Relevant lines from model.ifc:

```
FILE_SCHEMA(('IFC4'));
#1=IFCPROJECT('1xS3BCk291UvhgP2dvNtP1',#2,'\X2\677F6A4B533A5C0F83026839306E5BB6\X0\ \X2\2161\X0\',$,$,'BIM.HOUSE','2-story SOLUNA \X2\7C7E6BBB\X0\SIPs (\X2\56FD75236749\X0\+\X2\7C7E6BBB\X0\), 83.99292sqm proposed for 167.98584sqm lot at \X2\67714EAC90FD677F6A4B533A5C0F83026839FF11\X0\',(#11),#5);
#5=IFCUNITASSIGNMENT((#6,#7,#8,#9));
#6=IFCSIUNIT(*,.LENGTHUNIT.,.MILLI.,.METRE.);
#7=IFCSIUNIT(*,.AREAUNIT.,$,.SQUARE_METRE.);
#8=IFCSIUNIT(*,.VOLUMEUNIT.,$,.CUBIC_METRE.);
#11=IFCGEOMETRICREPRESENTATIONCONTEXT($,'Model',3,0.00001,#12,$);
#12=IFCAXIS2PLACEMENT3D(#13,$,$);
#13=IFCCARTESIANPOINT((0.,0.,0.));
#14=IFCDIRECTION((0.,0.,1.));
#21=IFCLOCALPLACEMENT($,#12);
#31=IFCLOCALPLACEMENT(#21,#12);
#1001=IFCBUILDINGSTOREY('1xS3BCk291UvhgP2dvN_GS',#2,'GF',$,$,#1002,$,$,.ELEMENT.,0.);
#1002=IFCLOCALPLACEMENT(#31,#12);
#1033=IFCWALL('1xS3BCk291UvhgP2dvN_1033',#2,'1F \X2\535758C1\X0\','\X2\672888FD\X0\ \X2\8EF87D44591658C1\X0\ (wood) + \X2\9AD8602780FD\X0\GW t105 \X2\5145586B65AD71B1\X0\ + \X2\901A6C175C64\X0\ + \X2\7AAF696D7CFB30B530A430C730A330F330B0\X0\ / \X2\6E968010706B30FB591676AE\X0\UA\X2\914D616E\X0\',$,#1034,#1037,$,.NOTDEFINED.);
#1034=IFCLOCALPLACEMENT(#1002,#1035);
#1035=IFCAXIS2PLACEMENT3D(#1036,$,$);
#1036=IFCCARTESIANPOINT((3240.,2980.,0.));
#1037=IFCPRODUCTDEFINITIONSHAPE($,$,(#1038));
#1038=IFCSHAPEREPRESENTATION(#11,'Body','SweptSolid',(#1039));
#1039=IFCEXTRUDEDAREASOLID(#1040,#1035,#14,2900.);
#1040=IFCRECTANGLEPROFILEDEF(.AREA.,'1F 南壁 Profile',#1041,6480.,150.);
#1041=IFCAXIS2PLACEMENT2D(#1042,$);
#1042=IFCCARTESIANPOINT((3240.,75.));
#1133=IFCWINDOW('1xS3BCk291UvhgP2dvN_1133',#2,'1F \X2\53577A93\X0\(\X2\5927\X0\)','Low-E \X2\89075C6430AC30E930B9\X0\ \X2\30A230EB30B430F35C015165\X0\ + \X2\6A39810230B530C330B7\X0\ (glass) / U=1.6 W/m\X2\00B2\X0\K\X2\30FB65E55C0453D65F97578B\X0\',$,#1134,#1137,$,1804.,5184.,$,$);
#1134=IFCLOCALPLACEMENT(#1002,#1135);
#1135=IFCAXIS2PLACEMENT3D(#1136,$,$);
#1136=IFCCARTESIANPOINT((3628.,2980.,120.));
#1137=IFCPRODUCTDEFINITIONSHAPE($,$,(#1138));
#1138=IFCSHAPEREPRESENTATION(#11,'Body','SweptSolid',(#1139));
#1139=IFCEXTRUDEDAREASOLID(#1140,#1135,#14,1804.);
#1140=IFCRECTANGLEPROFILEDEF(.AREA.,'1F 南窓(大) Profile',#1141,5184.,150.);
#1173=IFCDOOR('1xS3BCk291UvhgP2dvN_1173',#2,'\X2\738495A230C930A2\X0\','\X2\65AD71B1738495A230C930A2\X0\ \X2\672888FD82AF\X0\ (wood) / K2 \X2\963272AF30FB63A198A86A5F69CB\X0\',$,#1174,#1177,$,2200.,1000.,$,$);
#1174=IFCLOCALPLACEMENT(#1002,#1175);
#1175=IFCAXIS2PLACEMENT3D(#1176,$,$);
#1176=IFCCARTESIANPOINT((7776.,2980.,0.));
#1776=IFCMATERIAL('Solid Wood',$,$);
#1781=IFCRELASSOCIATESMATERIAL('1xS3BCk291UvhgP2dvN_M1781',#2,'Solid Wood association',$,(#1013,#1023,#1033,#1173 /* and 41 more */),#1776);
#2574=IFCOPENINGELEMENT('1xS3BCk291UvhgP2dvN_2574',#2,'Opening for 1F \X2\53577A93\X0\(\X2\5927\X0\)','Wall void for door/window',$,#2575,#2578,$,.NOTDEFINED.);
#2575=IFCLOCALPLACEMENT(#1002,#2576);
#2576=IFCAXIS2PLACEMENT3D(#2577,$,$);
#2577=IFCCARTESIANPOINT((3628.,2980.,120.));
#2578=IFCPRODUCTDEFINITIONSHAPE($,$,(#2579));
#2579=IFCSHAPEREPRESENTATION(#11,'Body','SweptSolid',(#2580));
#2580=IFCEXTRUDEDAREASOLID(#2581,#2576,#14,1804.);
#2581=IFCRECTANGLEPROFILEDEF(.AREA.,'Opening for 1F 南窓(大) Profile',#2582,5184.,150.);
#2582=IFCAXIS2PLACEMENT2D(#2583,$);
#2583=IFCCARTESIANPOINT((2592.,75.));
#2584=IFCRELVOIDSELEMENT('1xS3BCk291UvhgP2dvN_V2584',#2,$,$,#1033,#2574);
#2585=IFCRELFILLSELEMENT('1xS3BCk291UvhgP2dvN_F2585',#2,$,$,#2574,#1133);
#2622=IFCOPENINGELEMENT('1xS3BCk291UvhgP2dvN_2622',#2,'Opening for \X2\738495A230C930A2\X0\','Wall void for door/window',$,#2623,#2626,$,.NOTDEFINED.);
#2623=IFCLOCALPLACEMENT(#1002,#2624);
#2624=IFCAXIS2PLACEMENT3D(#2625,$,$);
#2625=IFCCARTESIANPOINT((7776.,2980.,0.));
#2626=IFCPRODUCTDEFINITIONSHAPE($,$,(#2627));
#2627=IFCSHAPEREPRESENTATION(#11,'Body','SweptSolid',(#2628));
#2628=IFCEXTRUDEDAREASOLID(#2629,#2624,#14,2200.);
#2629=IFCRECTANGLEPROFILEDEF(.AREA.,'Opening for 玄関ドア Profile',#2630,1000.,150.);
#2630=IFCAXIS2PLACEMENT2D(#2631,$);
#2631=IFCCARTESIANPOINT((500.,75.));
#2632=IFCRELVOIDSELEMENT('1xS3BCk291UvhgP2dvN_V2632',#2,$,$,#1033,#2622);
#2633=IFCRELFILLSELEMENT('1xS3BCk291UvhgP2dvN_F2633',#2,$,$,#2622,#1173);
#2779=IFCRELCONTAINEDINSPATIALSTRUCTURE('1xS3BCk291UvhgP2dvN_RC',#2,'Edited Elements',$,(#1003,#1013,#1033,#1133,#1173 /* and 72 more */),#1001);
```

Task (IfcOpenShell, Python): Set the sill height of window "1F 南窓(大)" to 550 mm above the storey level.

```python
import numpy as np
import ifcopenshell
import ifcopenshell.api.geometry
import ifcopenshell.geom
import ifcopenshell.util.element
import ifcopenshell.util.placement
import ifcopenshell.util.shape
import ifcopenshell.util.unit

model = ifcopenshell.open("model.ifc")
unit_scale = ifcopenshell.util.unit.calculate_unit_scale(model)

window = model.by_id(1133)
opening = window.FillsVoids[0].RelatingOpeningElement
storey = ifcopenshell.util.element.get_container(window, ifc_class="IfcBuildingStorey")
level = ifcopenshell.util.placement.get_local_placement(storey.ObjectPlacement)[2, 3]

# The opening's origin need not be at the sill, so measure its lowest point.
shape = ifcopenshell.geom.create_shape(ifcopenshell.geom.settings(), opening)
bottom = ifcopenshell.util.shape.get_shape_bottom_elevation(shape, shape.geometry) / unit_scale
dz = level + 0.55 / unit_scale - bottom

shift = np.array([0.0, 0.0, dz])
# The window is not placed relative to its opening, so move both.
for product in (opening, window):
    matrix = ifcopenshell.util.placement.get_local_placement(product.ObjectPlacement)
    matrix[:3, 3] += shift
    ifcopenshell.api.geometry.edit_object_placement(model, product=product, matrix=matrix, is_si=False)

print(f"moved by {dz * unit_scale:+.3f} m")

model.write("model_edited.ifc")
```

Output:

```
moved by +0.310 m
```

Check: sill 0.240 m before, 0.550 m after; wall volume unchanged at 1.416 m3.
